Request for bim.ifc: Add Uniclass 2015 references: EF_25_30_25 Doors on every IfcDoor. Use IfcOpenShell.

First a look at what the model holds.

```python
import ifcopenshell

model = ifcopenshell.open("bim.ifc")
print(model.schema)
print("classifications:", [c.Name for c in model.by_type("IfcClassification")])
for ifc_class in ("IfcDoor", "IfcRoof", "IfcStair", "IfcWall", "IfcWindow"):
    print(ifc_class, len(model.by_type(ifc_class)))
```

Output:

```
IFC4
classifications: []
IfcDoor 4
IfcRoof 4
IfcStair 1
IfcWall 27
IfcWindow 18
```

```python
import ifcopenshell
import ifcopenshell.api.classification

model = ifcopenshell.open("bim.ifc")

system = ifcopenshell.api.classification.add_classification(model, classification="Uniclass 2015")

codes = {
    "IfcDoor": ("EF_25_30_25", "Doors"),
}
for ifc_class, (code, name) in codes.items():
    products = model.by_type(ifc_class)
    ifcopenshell.api.classification.add_reference(
        model, products=products, classification=system, identification=code, name=name
    )
    print(code, len(products))

model.write("bim_v2.ifc")
```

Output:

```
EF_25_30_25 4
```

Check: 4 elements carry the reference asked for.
